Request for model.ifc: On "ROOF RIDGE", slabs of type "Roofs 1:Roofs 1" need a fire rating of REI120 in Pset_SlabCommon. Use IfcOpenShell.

First a look at what the model holds.

```python
import ifcopenshell
import ifcopenshell.util.element

model = ifcopenshell.open("model.ifc")
print(model.schema)
storey = next(s for s in model.by_type("IfcBuildingStorey") if s.Name == "ROOF RIDGE")
slabs = [e for e in ifcopenshell.util.element.get_decomposition(storey) if e.is_a("IfcSlab")]
seen = {}
for e in slabs:
    element_type = ifcopenshell.util.element.get_type(e)
    key = (element_type.Name if element_type != e and element_type else None, ifcopenshell.util.element.get_pset(e, "Pset_SlabCommon", "FireRating"))
    seen[key] = seen.get(key, 0) + 1
for (name, value), count in sorted(seen.items(), key=str):
    print(count, "x", name, "|", value)
```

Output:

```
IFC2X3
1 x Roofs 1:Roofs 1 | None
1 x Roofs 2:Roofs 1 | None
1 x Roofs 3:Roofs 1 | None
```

```python
import ifcopenshell
import ifcopenshell.api.pset
import ifcopenshell.util.element

model = ifcopenshell.open("model.ifc")

storey = next(s for s in model.by_type("IfcBuildingStorey") if s.Name == "ROOF RIDGE")
slabs = [e for e in ifcopenshell.util.element.get_decomposition(storey) if e.is_a("IfcSlab")]

count = 0
for e in slabs:
    element_type = ifcopenshell.util.element.get_type(e)
    if element_type in (None, e) or element_type.Name != "Roofs 1:Roofs 1":
        continue
    # add_pset returns the element's existing set when there is one.
    pset = ifcopenshell.api.pset.add_pset(model, product=e, name="Pset_SlabCommon")
    ifcopenshell.api.pset.edit_pset(model, pset=pset, properties={"FireRating": "REI120"})
    count += 1

print(count, "slabs updated")

model.write("model_v2.ifc")
```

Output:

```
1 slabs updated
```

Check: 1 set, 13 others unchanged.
